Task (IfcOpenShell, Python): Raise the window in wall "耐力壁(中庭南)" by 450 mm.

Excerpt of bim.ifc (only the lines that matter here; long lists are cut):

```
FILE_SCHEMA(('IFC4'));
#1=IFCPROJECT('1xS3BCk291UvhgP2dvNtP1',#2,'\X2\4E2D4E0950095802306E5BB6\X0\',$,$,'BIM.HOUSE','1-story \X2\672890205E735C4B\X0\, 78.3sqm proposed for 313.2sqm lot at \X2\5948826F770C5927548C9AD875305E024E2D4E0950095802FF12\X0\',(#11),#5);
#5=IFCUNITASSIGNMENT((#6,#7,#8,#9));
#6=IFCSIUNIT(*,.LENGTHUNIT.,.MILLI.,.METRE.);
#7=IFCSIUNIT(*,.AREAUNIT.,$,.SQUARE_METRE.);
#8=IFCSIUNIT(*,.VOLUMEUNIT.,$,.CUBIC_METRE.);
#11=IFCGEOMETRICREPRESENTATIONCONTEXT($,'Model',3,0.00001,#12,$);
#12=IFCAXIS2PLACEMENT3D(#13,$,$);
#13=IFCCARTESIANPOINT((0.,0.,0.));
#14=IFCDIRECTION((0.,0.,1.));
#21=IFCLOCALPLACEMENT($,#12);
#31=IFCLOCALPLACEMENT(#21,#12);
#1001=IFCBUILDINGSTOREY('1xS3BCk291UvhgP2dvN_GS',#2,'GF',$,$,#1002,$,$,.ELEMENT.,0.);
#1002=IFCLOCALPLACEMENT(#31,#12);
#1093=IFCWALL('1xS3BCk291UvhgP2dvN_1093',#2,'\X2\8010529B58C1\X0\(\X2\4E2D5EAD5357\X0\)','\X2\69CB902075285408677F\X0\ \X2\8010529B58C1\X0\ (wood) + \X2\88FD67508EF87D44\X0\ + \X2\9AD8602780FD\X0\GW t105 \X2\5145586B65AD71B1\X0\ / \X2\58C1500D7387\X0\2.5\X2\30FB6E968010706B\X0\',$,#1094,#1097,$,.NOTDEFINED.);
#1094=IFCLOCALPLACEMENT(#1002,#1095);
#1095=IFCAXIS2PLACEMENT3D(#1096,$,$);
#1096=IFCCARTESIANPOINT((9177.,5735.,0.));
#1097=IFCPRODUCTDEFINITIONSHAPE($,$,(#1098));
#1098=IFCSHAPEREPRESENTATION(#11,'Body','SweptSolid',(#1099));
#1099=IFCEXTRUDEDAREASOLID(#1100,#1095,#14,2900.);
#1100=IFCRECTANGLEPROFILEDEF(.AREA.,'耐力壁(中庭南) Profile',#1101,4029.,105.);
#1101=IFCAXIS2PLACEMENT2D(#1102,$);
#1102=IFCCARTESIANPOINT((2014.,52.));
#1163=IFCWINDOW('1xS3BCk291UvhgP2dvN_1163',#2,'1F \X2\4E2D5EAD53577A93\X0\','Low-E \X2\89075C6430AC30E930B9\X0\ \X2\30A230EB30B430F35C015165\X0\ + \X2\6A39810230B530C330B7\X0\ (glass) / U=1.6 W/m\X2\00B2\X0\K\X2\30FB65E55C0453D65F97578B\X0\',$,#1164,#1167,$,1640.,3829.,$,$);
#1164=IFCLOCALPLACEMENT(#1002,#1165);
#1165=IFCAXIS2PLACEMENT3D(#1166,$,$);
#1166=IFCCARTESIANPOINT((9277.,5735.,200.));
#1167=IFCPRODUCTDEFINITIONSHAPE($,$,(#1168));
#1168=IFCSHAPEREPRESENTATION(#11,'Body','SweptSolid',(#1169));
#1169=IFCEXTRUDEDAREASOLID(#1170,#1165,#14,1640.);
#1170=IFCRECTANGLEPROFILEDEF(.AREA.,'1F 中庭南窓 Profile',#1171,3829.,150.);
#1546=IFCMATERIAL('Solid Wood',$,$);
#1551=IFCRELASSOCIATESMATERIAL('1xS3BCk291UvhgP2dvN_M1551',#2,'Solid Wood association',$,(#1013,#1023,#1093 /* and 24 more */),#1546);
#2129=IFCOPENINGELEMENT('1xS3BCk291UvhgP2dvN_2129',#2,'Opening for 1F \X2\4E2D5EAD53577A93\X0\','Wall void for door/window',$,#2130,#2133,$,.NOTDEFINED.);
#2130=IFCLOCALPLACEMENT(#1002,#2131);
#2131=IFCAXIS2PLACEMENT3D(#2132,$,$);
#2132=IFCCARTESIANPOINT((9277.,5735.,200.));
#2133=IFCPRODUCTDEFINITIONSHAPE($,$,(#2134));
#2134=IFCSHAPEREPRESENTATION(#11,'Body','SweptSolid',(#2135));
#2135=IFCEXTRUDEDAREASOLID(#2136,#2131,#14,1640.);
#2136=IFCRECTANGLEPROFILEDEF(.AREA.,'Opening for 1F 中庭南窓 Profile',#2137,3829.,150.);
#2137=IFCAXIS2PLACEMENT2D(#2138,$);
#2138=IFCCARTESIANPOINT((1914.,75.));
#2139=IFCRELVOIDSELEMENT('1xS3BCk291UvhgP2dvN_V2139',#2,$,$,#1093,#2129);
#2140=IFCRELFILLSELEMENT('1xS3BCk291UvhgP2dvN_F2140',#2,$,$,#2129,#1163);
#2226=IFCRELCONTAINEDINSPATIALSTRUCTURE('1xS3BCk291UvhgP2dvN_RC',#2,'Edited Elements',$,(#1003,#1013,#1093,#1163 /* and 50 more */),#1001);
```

```python
import numpy as np
import ifcopenshell
import ifcopenshell.api.geometry
import ifcopenshell.util.placement
import ifcopenshell.util.unit

model = ifcopenshell.open("bim.ifc")
unit_scale = ifcopenshell.util.unit.calculate_unit_scale(model)

window = model.by_guid("1xS3BCk291UvhgP2dvN_1163")
opening = window.FillsVoids[0].RelatingOpeningElement
dz = 0.45 / unit_scale

shift = np.array([0.0, 0.0, dz])
# The window is not placed relative to its opening, so move both.
for product in (opening, window):
    matrix = ifcopenshell.util.placement.get_local_placement(product.ObjectPlacement)
    matrix[:3, 3] += shift
    ifcopenshell.api.geometry.edit_object_placement(model, product=product, matrix=matrix, is_si=False)

print(f"moved by {dz * unit_scale:+.3f} m")

model.write("bim_edited.ifc")
```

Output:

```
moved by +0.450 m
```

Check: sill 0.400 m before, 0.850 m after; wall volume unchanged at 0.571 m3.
